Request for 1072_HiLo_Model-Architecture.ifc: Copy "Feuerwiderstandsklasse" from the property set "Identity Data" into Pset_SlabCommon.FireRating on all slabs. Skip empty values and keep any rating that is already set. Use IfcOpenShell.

First a look at what the model holds.

```python
import ifcopenshell
import ifcopenshell.util.element

model = ifcopenshell.open("1072_HiLo_Model-Architecture.ifc")
print(model.schema)
slabs = model.by_type("IfcSlab")
print(len(slabs), "slabs")
for e in slabs[:8]:
    source = ifcopenshell.util.element.get_pset(e, "Identity Data", "Feuerwiderstandsklasse")
    target = ifcopenshell.util.element.get_pset(e, "Pset_SlabCommon", "FireRating")
    print(e.id(), repr(source), repr(target), sep=" | ")
```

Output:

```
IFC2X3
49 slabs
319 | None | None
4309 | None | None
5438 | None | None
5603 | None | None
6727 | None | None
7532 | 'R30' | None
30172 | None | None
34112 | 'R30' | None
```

```python
import ifcopenshell
import ifcopenshell.api.pset
import ifcopenshell.util.element

model = ifcopenshell.open("1072_HiLo_Model-Architecture.ifc")

count = 0
for e in model.by_type("IfcSlab"):
    value = ifcopenshell.util.element.get_pset(e, "Identity Data", "Feuerwiderstandsklasse")
    current = ifcopenshell.util.element.get_pset(e, "Pset_SlabCommon", "FireRating")
    if not value or not value.strip() or current:
        continue
    # add_pset returns the element's existing set when there is one.
    pset = ifcopenshell.api.pset.add_pset(model, product=e, name="Pset_SlabCommon")
    ifcopenshell.api.pset.edit_pset(model, pset=pset, properties={"FireRating": value})
    count += 1

print(count, "slabs updated")

model.write("1072_HiLo_Model-Architecture_rev.ifc")
```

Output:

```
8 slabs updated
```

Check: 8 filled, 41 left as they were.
